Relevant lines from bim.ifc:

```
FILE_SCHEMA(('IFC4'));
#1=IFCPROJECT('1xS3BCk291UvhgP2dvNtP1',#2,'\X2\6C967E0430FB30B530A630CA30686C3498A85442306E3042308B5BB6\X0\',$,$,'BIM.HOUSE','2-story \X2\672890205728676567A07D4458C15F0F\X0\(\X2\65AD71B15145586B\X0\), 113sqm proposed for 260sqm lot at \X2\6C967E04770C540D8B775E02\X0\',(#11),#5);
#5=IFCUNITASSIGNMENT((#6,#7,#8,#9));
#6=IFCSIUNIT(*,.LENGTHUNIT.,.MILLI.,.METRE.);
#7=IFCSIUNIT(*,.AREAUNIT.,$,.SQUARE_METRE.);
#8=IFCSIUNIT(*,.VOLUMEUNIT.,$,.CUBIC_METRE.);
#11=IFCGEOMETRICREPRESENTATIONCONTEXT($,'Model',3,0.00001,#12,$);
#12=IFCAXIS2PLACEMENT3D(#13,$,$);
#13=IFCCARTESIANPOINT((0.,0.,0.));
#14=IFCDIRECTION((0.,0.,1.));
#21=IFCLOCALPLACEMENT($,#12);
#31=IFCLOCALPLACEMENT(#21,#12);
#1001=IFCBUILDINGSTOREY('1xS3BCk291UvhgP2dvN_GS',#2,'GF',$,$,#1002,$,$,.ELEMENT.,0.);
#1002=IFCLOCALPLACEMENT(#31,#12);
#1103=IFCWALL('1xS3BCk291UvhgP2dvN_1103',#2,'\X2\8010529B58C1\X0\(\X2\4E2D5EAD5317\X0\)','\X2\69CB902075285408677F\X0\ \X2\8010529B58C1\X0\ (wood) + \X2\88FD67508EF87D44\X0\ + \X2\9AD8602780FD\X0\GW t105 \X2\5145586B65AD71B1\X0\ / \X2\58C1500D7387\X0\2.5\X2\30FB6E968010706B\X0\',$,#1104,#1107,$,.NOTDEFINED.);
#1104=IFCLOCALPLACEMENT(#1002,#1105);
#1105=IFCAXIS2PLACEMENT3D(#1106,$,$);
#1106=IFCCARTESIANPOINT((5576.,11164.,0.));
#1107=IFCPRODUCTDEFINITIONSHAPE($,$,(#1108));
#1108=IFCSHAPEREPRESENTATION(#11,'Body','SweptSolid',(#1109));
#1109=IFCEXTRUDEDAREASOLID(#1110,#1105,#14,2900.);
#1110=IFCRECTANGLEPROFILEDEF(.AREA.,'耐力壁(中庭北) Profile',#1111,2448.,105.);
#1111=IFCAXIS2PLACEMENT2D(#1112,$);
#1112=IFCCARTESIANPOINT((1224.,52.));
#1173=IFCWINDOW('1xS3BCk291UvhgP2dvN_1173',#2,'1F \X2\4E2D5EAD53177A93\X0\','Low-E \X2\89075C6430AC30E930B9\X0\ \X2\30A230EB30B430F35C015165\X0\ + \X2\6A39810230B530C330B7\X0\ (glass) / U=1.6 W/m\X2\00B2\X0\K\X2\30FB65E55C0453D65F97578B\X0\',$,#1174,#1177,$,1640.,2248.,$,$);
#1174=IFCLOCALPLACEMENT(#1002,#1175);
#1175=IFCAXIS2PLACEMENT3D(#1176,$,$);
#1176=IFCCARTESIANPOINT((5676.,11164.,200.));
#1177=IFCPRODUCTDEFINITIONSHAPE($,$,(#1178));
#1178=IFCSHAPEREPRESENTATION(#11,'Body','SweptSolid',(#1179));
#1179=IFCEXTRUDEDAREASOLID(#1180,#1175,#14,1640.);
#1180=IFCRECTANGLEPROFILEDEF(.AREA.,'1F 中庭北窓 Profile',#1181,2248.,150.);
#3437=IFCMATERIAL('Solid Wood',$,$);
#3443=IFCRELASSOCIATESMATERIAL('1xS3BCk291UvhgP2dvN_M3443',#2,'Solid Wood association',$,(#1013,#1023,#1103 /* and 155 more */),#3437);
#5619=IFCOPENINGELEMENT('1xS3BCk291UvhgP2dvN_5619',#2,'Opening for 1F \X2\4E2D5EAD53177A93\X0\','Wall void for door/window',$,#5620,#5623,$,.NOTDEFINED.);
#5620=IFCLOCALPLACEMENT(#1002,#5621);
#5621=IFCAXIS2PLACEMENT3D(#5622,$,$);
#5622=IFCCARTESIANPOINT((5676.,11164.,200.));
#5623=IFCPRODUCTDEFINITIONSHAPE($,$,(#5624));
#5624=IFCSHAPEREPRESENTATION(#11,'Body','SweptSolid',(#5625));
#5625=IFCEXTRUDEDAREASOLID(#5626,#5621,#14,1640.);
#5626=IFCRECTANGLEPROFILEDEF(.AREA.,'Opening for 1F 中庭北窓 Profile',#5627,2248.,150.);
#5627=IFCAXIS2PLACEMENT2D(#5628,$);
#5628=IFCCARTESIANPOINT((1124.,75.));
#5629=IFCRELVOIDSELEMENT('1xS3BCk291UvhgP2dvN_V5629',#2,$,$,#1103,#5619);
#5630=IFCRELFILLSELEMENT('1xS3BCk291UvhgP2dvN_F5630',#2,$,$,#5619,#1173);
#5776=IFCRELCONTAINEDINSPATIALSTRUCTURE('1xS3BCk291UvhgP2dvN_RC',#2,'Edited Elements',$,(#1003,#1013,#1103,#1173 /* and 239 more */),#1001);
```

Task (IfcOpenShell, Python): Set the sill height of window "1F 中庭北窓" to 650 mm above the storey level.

```python
import numpy as np
import ifcopenshell
import ifcopenshell.api.geometry
import ifcopenshell.geom
import ifcopenshell.util.element
import ifcopenshell.util.placement
import ifcopenshell.util.shape
import ifcopenshell.util.unit

model = ifcopenshell.open("bim.ifc")
unit_scale = ifcopenshell.util.unit.calculate_unit_scale(model)

window = model.by_guid("1xS3BCk291UvhgP2dvN_1173")
opening = window.FillsVoids[0].RelatingOpeningElement
storey = ifcopenshell.util.element.get_container(window, ifc_class="IfcBuildingStorey")
level = ifcopenshell.util.placement.get_local_placement(storey.ObjectPlacement)[2, 3]

# The opening's origin need not be at the sill, so measure its lowest point.
shape = ifcopenshell.geom.create_shape(ifcopenshell.geom.settings(), opening)
bottom = ifcopenshell.util.shape.get_shape_bottom_elevation(shape, shape.geometry) / unit_scale
dz = level + 650.0 - bottom

shift = np.array([0.0, 0.0, dz])
# The window is not placed relative to its opening, so move both.
for product in (opening, window):
    matrix = ifcopenshell.util.placement.get_local_placement(product.ObjectPlacement)
    matrix[:3, 3] += shift
    ifcopenshell.api.geometry.edit_object_placement(model, product=product, matrix=matrix, is_si=False)

print(f"moved by {dz * unit_scale:+.3f} m")

model.write("bim_rev.ifc")
```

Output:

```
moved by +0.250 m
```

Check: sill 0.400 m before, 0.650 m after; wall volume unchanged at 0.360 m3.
